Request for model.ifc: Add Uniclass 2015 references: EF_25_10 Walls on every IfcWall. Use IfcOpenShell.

First a look at what the model holds.

```python
import ifcopenshell

model = ifcopenshell.open("model.ifc")
print(model.schema)
print("classifications:", [c.Name for c in model.by_type("IfcClassification")])
for ifc_class in ("IfcDoor", "IfcRoof", "IfcStair", "IfcWall", "IfcWindow"):
    print(ifc_class, len(model.by_type(ifc_class)))
```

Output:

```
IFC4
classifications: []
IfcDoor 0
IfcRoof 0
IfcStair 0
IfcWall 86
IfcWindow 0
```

```python
import ifcopenshell
import ifcopenshell.api.classification

model = ifcopenshell.open("model.ifc")

system = ifcopenshell.api.classification.add_classification(model, classification="Uniclass 2015")

codes = {
    "IfcWall": ("EF_25_10", "Walls"),
}
for ifc_class, (code, name) in codes.items():
    products = model.by_type(ifc_class)
    ifcopenshell.api.classification.add_reference(
        model, products=products, classification=system, identification=code, name=name
    )
    print(code, len(products))

model.write("model_rev.ifc")
```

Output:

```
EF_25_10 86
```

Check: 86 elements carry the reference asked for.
